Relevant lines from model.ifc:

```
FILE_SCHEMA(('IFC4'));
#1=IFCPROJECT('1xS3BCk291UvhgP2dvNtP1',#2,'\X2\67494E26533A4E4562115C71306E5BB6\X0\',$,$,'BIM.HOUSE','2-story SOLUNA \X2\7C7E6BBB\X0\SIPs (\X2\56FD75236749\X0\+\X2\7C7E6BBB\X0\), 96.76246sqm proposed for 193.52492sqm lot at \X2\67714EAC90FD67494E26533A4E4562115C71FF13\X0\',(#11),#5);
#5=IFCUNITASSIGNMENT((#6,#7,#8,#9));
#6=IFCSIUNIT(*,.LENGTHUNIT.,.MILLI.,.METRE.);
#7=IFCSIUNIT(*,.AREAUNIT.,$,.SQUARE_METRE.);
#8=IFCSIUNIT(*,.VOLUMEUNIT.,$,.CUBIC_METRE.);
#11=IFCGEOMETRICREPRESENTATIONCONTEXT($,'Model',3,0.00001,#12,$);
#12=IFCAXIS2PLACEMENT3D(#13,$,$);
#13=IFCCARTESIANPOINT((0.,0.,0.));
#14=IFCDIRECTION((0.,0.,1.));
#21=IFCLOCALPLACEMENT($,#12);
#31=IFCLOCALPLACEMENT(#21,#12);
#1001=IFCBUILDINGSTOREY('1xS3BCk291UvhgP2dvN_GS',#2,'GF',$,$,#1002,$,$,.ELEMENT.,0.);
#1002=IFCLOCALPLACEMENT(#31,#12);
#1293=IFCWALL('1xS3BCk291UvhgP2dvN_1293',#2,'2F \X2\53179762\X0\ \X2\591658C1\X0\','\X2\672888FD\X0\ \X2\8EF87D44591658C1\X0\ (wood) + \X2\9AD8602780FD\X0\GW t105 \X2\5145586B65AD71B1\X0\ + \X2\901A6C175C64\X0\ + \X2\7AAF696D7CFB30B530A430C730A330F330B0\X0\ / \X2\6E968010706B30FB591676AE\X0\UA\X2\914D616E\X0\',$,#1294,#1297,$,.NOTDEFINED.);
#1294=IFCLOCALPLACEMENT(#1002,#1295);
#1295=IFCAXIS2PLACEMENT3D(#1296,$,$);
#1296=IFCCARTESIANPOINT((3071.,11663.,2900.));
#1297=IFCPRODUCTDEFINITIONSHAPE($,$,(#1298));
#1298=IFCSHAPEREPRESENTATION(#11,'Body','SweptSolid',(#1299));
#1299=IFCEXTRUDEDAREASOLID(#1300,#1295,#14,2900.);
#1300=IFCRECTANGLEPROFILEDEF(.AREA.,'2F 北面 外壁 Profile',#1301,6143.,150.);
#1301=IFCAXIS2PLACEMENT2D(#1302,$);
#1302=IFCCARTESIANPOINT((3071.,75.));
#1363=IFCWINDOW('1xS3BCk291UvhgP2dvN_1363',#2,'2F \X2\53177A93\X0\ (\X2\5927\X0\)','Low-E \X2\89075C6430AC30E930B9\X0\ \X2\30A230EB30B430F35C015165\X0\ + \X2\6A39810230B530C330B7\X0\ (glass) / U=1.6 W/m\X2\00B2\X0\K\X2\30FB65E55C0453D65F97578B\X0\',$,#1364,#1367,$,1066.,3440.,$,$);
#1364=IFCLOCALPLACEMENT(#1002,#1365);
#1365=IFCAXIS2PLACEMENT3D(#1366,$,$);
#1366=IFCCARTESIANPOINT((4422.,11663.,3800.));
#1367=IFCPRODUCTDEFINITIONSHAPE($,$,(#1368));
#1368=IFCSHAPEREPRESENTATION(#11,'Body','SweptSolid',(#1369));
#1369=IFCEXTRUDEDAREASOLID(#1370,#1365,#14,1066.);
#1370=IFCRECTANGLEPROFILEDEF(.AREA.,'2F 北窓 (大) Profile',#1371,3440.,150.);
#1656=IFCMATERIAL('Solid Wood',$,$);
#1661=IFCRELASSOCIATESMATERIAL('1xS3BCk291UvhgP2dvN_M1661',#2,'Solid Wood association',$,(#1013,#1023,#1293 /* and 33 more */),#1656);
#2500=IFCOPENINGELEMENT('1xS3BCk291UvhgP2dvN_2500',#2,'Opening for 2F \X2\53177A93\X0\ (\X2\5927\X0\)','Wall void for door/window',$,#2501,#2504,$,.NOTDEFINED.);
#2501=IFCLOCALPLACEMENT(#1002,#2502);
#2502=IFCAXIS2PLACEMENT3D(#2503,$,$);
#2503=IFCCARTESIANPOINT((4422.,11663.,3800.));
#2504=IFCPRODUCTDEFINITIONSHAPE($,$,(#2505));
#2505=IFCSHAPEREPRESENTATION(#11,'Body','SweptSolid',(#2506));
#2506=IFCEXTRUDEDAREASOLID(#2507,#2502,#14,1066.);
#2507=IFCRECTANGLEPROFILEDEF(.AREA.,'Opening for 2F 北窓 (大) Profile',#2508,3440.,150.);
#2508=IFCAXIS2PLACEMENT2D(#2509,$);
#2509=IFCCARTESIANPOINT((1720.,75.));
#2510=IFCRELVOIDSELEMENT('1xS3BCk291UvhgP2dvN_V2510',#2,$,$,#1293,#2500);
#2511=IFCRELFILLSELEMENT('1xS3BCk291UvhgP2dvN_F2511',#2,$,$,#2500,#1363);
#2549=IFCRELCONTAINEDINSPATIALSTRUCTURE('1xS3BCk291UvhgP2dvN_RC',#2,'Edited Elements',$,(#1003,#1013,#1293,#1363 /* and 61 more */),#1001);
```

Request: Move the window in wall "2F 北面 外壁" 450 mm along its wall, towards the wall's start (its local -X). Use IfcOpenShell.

```python
import ifcopenshell
import ifcopenshell.api.geometry
import ifcopenshell.util.placement

model = ifcopenshell.open("model.ifc")

window = model.by_guid("1xS3BCk291UvhgP2dvN_1363")
opening = window.FillsVoids[0].RelatingOpeningElement
wall = opening.VoidsElements[0].RelatingBuildingElement

wall_matrix = ifcopenshell.util.placement.get_local_placement(wall.ObjectPlacement)
shift = wall_matrix[:3, 0] * -450.0
before = ifcopenshell.util.placement.get_local_placement(window.ObjectPlacement)[:3, 3].copy()

# The window is not placed relative to its opening, so move both.
for product in (opening, window):
    matrix = ifcopenshell.util.placement.get_local_placement(product.ObjectPlacement)
    matrix[:3, 3] += shift
    ifcopenshell.api.geometry.edit_object_placement(model, product=product, matrix=matrix, is_si=False)

after = ifcopenshell.util.placement.get_local_placement(window.ObjectPlacement)[:3, 3]
print("window moved by", (after - before).round(3) + 0.0)

model.write("model-out.ifc")
```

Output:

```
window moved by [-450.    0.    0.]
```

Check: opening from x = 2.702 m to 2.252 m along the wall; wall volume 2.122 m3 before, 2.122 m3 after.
